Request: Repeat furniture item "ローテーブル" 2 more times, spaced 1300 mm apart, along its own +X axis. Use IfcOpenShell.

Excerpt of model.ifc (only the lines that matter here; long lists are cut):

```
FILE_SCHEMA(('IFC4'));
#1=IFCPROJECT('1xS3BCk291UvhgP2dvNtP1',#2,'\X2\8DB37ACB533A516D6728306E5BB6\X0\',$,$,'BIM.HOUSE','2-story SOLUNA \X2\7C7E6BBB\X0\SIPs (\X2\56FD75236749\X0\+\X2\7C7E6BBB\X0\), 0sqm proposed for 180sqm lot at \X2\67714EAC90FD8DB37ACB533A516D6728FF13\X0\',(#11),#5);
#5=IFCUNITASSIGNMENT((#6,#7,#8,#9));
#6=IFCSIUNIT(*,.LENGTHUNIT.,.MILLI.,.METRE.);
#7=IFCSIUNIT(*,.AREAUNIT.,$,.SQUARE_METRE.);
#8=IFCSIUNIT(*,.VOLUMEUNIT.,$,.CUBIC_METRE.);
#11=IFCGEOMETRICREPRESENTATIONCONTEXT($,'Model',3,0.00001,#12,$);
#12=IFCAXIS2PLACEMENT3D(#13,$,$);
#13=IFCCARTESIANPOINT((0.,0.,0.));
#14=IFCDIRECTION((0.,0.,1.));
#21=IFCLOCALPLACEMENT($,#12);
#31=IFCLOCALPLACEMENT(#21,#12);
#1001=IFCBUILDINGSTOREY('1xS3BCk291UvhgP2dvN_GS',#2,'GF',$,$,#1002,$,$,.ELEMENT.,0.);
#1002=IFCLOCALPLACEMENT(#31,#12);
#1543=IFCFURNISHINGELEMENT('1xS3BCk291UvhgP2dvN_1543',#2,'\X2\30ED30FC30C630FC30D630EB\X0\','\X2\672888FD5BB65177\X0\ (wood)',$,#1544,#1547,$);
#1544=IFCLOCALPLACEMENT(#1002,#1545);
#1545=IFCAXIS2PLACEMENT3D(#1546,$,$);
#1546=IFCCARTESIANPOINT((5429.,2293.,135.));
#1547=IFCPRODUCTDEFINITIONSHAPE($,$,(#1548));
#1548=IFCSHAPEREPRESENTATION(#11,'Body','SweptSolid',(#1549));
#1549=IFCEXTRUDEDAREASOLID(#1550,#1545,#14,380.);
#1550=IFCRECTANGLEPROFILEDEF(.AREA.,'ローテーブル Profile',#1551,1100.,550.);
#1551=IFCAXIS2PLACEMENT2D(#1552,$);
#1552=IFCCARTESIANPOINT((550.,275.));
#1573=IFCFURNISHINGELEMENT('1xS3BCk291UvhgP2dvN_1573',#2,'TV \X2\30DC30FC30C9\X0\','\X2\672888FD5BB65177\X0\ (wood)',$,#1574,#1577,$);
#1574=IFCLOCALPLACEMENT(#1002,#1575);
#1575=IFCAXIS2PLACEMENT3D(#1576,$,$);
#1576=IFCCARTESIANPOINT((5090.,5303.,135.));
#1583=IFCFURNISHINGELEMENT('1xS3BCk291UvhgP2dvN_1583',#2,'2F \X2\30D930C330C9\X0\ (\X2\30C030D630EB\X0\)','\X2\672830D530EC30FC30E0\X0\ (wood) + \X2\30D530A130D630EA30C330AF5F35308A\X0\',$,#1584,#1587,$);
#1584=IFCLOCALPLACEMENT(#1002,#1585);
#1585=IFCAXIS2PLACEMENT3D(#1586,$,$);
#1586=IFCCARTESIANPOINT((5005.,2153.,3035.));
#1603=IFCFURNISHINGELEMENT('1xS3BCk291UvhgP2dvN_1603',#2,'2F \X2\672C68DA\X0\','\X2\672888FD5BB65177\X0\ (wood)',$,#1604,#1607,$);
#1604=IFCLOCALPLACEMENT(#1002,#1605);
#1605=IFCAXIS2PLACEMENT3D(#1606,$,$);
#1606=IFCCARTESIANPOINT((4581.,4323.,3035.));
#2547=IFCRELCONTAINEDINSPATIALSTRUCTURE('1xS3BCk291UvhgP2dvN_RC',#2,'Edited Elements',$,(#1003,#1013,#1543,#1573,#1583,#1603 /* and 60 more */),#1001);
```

```python
import ifcopenshell
import ifcopenshell.api.geometry
import ifcopenshell.api.root
import ifcopenshell.util.element
import ifcopenshell.util.placement

model = ifcopenshell.open("model.ifc")


def reuse_history(source, copy):
    """copy_class also copies each property set's owner history, people and application; keep the originals."""
    for rel in copy.IsDefinedBy:
        if rel.is_a("IfcRelDefinesByProperties") and (history := rel.RelatingPropertyDefinition.OwnerHistory):
            rel.RelatingPropertyDefinition.OwnerHistory = source.OwnerHistory
            ifcopenshell.util.element.remove_deep2(model, history)


source = model.by_id(1543)
base = ifcopenshell.util.placement.get_local_placement(source.ObjectPlacement)
step = base[:3, 0] * 1300.0

for i in range(1, 3):
    copy = ifcopenshell.api.root.copy_class(model, product=source)
    copy.Representation = ifcopenshell.util.element.copy_deep(
        model, source.Representation, exclude=["IfcGeometricRepresentationContext", "IfcRepresentationMap"]
    )
    reuse_history(source, copy)
    matrix = base.copy()
    matrix[:3, 3] += i * step
    print("added at", matrix[:3, 3].round(3) + 0.0)
    ifcopenshell.api.geometry.edit_object_placement(model, product=copy, matrix=matrix, is_si=False)

model.write("model_rev.ifc")
```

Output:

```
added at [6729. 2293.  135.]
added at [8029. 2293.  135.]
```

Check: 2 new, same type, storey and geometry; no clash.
